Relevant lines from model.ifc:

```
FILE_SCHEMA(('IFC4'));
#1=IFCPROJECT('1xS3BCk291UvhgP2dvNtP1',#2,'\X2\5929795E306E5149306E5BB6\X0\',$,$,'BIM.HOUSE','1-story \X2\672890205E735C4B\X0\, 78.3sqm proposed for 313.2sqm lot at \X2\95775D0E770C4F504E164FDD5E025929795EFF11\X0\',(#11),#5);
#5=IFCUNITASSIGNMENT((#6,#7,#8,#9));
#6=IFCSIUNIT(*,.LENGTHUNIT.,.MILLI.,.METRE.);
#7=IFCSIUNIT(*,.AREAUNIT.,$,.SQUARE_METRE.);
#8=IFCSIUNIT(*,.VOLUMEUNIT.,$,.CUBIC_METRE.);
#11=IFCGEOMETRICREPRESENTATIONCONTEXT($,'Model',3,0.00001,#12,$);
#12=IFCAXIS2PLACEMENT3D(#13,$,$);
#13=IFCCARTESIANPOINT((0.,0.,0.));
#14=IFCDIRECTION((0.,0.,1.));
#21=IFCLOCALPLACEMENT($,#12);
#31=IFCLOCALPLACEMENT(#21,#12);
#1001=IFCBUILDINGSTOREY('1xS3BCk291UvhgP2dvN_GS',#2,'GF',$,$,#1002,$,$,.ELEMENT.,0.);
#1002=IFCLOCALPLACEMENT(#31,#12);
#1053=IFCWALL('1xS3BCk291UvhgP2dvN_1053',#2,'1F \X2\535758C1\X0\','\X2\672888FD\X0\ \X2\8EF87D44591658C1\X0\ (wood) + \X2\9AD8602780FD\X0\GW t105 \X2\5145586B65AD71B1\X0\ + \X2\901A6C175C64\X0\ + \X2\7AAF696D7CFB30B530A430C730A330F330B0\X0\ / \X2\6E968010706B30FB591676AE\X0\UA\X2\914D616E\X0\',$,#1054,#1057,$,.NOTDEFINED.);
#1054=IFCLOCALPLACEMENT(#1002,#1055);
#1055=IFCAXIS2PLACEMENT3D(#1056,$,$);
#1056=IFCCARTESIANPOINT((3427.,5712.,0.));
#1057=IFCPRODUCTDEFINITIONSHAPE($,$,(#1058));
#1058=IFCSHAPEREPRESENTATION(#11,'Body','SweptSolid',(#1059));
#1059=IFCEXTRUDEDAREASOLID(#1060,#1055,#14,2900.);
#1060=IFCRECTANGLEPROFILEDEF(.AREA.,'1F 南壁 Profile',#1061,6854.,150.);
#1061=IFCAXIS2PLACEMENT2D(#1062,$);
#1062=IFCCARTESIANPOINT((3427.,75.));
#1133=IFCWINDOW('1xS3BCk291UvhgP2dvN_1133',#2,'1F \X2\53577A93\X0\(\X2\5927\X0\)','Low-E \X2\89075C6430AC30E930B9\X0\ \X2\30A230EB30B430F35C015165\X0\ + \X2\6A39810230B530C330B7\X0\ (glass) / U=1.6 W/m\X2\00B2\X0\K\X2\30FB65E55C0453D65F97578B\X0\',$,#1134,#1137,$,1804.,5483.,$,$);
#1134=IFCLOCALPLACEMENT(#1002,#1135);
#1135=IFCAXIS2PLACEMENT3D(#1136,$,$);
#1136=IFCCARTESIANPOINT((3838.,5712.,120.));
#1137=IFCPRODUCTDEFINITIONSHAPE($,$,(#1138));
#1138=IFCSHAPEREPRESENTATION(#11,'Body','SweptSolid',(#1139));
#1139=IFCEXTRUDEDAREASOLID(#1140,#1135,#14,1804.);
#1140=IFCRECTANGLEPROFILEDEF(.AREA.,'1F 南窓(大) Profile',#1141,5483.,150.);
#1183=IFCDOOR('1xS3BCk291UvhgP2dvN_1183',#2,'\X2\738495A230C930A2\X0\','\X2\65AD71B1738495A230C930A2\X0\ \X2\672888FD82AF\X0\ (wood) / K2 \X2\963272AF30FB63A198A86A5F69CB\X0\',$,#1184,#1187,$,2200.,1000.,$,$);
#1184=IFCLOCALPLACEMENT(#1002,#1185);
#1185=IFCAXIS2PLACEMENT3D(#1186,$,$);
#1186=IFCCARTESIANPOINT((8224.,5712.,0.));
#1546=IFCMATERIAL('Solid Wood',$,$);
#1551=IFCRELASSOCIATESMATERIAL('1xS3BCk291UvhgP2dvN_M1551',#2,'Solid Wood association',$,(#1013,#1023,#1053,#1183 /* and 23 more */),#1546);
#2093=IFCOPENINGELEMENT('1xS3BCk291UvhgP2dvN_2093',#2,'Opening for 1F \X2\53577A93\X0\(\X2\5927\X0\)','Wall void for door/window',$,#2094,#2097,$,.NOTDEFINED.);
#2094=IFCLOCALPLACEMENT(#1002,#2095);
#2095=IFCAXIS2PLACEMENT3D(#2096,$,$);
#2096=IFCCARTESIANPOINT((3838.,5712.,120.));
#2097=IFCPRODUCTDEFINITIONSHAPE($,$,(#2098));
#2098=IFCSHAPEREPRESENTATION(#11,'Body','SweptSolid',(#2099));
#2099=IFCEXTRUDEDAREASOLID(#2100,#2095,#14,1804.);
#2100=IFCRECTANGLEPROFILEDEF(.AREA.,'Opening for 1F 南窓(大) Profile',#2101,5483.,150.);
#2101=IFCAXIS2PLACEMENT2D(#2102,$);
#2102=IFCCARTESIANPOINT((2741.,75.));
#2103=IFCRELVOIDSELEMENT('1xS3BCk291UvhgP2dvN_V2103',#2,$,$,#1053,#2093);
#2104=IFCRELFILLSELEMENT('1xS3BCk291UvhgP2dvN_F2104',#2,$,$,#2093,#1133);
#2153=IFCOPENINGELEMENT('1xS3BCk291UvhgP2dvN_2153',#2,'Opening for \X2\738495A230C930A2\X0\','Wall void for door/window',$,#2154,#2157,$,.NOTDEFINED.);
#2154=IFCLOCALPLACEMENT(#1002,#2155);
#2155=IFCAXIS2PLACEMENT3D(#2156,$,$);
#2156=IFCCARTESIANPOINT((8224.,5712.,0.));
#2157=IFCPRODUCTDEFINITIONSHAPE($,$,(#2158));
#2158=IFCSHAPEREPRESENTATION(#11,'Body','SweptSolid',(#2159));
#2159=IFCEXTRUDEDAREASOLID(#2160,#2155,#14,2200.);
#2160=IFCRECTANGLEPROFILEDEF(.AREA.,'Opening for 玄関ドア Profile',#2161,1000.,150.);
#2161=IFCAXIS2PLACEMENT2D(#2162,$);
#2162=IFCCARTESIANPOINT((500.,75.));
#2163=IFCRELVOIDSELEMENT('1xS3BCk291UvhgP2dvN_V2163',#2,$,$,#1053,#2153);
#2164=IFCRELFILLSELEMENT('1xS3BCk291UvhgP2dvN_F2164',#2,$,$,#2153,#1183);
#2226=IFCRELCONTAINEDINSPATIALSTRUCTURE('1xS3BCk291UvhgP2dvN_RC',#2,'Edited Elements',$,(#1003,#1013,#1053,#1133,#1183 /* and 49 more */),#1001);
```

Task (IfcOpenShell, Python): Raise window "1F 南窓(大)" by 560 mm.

```python
import numpy as np
import ifcopenshell
import ifcopenshell.api.geometry
import ifcopenshell.util.placement
import ifcopenshell.util.unit

model = ifcopenshell.open("model.ifc")
unit_scale = ifcopenshell.util.unit.calculate_unit_scale(model)

window = model.by_guid("1xS3BCk291UvhgP2dvN_1133")
opening = window.FillsVoids[0].RelatingOpeningElement
dz = 0.56 / unit_scale

shift = np.array([0.0, 0.0, dz])
# The window is not placed relative to its opening, so move both.
for product in (opening, window):
    matrix = ifcopenshell.util.placement.get_local_placement(product.ObjectPlacement)
    matrix[:3, 3] += shift
    ifcopenshell.api.geometry.edit_object_placement(model, product=product, matrix=matrix, is_si=False)

print(f"moved by {dz * unit_scale:+.3f} m")

model.write("model-out.ifc")
```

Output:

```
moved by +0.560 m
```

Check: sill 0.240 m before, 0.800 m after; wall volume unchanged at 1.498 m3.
